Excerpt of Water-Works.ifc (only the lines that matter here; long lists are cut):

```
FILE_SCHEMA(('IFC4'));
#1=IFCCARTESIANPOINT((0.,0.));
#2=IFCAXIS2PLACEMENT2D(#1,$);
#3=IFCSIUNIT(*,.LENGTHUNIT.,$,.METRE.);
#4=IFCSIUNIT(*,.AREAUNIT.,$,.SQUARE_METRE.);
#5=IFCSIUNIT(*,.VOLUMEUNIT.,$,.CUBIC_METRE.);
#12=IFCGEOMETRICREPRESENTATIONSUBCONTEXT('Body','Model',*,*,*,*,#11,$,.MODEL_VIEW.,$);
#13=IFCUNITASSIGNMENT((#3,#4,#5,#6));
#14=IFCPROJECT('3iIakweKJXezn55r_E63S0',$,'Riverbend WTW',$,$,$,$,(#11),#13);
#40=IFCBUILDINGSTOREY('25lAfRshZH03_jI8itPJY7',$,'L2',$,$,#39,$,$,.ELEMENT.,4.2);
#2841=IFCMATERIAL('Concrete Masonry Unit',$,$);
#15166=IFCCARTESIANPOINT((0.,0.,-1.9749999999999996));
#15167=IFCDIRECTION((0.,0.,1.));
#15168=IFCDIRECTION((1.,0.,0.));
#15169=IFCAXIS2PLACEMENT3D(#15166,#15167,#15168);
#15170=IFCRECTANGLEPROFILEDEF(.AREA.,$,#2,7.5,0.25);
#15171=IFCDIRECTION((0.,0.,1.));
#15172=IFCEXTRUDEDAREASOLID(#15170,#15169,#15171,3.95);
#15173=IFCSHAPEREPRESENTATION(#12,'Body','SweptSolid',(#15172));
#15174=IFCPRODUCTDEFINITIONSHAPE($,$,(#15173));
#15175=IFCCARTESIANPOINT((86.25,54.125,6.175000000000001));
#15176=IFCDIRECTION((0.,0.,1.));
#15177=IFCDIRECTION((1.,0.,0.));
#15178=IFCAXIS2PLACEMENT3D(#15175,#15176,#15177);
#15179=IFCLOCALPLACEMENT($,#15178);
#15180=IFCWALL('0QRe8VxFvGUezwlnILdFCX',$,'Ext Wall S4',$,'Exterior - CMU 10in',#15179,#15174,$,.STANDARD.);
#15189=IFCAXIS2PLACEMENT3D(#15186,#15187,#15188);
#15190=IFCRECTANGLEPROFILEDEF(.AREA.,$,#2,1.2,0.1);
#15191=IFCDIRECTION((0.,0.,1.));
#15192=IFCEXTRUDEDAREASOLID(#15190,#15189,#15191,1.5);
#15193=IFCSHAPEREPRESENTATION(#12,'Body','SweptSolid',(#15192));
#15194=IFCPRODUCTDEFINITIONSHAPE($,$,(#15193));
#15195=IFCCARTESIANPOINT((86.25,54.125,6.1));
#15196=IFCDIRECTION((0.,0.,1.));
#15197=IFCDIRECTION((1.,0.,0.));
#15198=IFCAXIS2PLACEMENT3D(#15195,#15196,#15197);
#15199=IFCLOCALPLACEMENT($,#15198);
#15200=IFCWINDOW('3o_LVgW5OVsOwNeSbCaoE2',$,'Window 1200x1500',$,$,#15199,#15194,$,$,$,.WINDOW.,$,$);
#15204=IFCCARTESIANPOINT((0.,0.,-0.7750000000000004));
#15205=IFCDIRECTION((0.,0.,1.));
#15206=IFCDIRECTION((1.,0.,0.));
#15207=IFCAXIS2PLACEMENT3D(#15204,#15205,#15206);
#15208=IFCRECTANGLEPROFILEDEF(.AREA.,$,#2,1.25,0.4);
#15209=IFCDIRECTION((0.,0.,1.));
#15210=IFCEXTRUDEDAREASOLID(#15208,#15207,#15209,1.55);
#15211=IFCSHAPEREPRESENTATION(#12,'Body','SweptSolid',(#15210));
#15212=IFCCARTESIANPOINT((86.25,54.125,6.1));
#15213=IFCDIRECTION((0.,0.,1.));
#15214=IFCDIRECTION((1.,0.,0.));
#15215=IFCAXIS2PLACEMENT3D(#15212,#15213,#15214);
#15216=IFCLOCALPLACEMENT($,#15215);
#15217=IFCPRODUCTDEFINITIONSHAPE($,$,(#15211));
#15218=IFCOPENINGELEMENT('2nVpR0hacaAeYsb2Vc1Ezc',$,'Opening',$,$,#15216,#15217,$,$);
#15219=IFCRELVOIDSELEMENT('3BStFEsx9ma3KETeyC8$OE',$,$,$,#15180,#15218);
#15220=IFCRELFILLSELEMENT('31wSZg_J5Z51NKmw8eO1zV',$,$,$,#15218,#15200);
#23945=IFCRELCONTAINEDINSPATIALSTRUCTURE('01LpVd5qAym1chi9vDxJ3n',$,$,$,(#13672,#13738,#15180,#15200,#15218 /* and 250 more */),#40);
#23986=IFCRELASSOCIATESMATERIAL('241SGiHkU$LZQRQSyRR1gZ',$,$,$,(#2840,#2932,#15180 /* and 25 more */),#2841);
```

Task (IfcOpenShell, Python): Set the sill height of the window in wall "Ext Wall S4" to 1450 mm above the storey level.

```python
import numpy as np
import ifcopenshell
import ifcopenshell.api.geometry
import ifcopenshell.geom
import ifcopenshell.util.element
import ifcopenshell.util.placement
import ifcopenshell.util.shape
import ifcopenshell.util.unit

model = ifcopenshell.open("Water-Works.ifc")
unit_scale = ifcopenshell.util.unit.calculate_unit_scale(model)

window = model.by_id(15200)
opening = window.FillsVoids[0].RelatingOpeningElement
storey = ifcopenshell.util.element.get_container(window, ifc_class="IfcBuildingStorey")
level = ifcopenshell.util.placement.get_local_placement(storey.ObjectPlacement)[2, 3]

# The opening's origin need not be at the sill, so measure its lowest point.
shape = ifcopenshell.geom.create_shape(ifcopenshell.geom.settings(), opening)
bottom = ifcopenshell.util.shape.get_shape_bottom_elevation(shape, shape.geometry) / unit_scale
dz = level + 1.45 / unit_scale - bottom

shift = np.array([0.0, 0.0, dz])
# The window is not placed relative to its opening, so move both.
for product in (opening, window):
    matrix = ifcopenshell.util.placement.get_local_placement(product.ObjectPlacement)
    matrix[:3, 3] += shift
    ifcopenshell.api.geometry.edit_object_placement(model, product=product, matrix=matrix, is_si=False)

print(f"moved by {dz * unit_scale:+.3f} m")

model.write("Water-Works-out.ifc")
```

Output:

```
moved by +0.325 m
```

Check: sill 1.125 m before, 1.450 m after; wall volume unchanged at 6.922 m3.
